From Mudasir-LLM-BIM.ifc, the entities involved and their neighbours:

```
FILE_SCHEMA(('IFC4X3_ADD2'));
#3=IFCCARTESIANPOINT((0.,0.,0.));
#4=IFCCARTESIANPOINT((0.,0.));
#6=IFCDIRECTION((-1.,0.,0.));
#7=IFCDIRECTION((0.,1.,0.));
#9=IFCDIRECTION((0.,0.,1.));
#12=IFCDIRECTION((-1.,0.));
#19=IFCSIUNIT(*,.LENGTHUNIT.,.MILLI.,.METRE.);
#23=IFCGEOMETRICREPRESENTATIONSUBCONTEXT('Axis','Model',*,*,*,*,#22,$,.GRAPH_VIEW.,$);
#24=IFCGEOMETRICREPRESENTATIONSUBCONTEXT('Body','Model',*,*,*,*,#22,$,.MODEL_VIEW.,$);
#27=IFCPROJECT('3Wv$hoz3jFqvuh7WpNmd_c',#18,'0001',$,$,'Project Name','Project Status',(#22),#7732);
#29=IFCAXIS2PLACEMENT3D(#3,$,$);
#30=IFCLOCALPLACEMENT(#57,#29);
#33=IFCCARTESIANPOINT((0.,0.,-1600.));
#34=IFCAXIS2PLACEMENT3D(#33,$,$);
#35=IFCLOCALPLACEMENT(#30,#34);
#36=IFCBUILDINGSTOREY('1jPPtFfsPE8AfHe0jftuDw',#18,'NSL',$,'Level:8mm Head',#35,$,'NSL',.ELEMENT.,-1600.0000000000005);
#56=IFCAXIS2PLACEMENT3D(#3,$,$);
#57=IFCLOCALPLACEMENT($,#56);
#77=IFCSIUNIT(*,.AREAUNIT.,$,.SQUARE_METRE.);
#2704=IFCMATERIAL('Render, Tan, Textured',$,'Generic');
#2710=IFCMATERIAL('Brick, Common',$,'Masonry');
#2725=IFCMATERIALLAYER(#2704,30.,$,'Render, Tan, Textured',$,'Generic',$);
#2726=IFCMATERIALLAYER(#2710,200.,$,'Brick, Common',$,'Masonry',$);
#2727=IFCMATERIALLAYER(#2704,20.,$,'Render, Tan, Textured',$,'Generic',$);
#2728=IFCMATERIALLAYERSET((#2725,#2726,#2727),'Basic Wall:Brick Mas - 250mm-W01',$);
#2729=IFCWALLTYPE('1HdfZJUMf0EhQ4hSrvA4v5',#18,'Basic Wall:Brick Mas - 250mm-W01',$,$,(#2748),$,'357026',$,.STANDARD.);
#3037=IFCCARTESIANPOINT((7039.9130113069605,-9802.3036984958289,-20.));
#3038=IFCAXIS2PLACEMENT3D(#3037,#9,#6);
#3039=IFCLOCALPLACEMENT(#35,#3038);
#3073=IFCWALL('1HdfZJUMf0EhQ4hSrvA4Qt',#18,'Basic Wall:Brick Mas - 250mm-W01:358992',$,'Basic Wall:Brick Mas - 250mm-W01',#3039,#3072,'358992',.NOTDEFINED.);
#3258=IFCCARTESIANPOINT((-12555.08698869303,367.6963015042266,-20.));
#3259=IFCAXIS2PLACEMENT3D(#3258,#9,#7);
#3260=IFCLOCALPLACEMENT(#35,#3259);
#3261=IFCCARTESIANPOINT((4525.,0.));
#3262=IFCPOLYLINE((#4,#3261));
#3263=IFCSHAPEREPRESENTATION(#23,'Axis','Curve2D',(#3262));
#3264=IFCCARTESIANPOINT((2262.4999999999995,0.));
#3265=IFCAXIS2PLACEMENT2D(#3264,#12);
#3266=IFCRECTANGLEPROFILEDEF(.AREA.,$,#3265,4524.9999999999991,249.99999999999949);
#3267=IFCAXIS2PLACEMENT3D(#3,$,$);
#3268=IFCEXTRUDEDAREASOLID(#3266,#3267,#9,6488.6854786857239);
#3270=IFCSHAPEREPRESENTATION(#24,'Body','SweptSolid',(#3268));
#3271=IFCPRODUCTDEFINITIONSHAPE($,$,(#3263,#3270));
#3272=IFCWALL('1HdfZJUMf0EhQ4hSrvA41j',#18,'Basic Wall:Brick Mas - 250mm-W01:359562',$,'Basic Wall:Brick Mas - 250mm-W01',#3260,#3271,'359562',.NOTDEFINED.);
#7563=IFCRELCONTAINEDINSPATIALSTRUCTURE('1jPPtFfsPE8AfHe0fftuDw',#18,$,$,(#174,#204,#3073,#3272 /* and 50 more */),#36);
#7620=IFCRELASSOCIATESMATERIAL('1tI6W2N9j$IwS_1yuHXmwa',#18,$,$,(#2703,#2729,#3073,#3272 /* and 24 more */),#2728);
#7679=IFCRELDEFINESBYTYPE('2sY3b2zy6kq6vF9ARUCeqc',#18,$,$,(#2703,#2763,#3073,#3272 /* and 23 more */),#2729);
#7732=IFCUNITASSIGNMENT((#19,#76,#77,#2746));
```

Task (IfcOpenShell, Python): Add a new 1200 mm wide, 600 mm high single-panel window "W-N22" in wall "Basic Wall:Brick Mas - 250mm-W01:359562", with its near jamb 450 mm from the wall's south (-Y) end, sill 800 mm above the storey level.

```python
import numpy as np
import ifcopenshell
import ifcopenshell.api.feature
import ifcopenshell.api.geometry
import ifcopenshell.api.root
import ifcopenshell.api.spatial
import ifcopenshell.geom
import ifcopenshell.util.element
import ifcopenshell.util.placement
import ifcopenshell.util.representation
import ifcopenshell.util.shape
import ifcopenshell.util.unit

model = ifcopenshell.open("Mudasir-LLM-BIM.ifc")
unit_scale = ifcopenshell.util.unit.calculate_unit_scale(model)
settings = ifcopenshell.geom.settings()


def volume(element):
    """Net volume in cubic metres, openings subtracted."""
    shape = ifcopenshell.geom.create_shape(settings, element)
    return ifcopenshell.util.shape.get_volume(shape.geometry)


wall = model.by_guid("1HdfZJUMf0EhQ4hSrvA41j")
storey = ifcopenshell.util.element.get_container(wall, ifc_class="IfcBuildingStorey")
context = ifcopenshell.util.representation.get_context(model, "Model", "Body", "MODEL_VIEW")
before = volume(wall)

width, height, from_end, sill = 1.2, 0.6, 0.45, 0.8  # metres

# The wall runs along its own X axis, and the end named is its -X end.
wall_shape = ifcopenshell.geom.create_shape(settings, wall)
x, y, z = ifcopenshell.util.shape.get_vertices(wall_shape.geometry).T
start = x.min() + from_end
face, thickness = float(y.min()), float(y.max() - y.min())
wall_matrix = ifcopenshell.util.placement.get_local_placement(wall.ObjectPlacement)
level = ifcopenshell.util.placement.get_local_placement(storey.ObjectPlacement)[2, 3]


def in_wall(x, y):
    """Placement at x, y metres in the wall's axes, at sill height."""
    matrix = wall_matrix.copy()
    matrix[:, 3] = wall_matrix @ np.array([x / unit_scale, y / unit_scale, 0.0, 1.0])
    matrix[2, 3] = level + sill / unit_scale
    return matrix


# Opening: a box that overshoots both wall faces by 50 mm.
opening = ifcopenshell.api.root.create_entity(model, ifc_class="IfcOpeningElement", predefined_type="OPENING")
box = ifcopenshell.api.geometry.add_wall_representation(
    model, context=context, length=width, height=height, thickness=thickness + 0.1
)
ifcopenshell.api.geometry.assign_representation(model, product=opening, representation=box)
ifcopenshell.api.geometry.edit_object_placement(model, product=opening, matrix=in_wall(start, face - 0.05), is_si=False)
ifcopenshell.api.feature.add_feature(model, feature=opening, element=wall)

window = ifcopenshell.api.root.create_entity(model, ifc_class="IfcWindow", name="W-N22", predefined_type="WINDOW")
window.OverallWidth, window.OverallHeight = width / unit_scale, height / unit_scale
window.PartitioningType = "SINGLE_PANEL"
body = ifcopenshell.api.geometry.add_window_representation(
    model,
    context=context,
    overall_width=window.OverallWidth,
    overall_height=window.OverallHeight,
    partition_type="SINGLE_PANEL",
)
ifcopenshell.api.geometry.assign_representation(model, product=window, representation=body)
ifcopenshell.api.spatial.assign_container(model, products=[window], relating_structure=storey)
ifcopenshell.api.feature.add_filling(model, opening=opening, element=window)

# Centre the window in the wall's thickness.
ifcopenshell.api.geometry.edit_object_placement(model, product=window, matrix=in_wall(start, face), is_si=False)
window_shape = ifcopenshell.geom.create_shape(settings, window)
depth = ifcopenshell.util.shape.get_vertices(window_shape.geometry)[:, 1]
offset = face + thickness / 2 - (depth.min() + depth.max()) / 2
ifcopenshell.api.geometry.edit_object_placement(model, product=window, matrix=in_wall(start, offset), is_si=False)

after = volume(wall)

print(f"wall volume {before:.3f} -> {after:.3f} m3")

model.write("Mudasir-LLM-BIM_edited.ifc")
```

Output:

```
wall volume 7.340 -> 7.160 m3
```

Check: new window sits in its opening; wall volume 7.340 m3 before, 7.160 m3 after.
